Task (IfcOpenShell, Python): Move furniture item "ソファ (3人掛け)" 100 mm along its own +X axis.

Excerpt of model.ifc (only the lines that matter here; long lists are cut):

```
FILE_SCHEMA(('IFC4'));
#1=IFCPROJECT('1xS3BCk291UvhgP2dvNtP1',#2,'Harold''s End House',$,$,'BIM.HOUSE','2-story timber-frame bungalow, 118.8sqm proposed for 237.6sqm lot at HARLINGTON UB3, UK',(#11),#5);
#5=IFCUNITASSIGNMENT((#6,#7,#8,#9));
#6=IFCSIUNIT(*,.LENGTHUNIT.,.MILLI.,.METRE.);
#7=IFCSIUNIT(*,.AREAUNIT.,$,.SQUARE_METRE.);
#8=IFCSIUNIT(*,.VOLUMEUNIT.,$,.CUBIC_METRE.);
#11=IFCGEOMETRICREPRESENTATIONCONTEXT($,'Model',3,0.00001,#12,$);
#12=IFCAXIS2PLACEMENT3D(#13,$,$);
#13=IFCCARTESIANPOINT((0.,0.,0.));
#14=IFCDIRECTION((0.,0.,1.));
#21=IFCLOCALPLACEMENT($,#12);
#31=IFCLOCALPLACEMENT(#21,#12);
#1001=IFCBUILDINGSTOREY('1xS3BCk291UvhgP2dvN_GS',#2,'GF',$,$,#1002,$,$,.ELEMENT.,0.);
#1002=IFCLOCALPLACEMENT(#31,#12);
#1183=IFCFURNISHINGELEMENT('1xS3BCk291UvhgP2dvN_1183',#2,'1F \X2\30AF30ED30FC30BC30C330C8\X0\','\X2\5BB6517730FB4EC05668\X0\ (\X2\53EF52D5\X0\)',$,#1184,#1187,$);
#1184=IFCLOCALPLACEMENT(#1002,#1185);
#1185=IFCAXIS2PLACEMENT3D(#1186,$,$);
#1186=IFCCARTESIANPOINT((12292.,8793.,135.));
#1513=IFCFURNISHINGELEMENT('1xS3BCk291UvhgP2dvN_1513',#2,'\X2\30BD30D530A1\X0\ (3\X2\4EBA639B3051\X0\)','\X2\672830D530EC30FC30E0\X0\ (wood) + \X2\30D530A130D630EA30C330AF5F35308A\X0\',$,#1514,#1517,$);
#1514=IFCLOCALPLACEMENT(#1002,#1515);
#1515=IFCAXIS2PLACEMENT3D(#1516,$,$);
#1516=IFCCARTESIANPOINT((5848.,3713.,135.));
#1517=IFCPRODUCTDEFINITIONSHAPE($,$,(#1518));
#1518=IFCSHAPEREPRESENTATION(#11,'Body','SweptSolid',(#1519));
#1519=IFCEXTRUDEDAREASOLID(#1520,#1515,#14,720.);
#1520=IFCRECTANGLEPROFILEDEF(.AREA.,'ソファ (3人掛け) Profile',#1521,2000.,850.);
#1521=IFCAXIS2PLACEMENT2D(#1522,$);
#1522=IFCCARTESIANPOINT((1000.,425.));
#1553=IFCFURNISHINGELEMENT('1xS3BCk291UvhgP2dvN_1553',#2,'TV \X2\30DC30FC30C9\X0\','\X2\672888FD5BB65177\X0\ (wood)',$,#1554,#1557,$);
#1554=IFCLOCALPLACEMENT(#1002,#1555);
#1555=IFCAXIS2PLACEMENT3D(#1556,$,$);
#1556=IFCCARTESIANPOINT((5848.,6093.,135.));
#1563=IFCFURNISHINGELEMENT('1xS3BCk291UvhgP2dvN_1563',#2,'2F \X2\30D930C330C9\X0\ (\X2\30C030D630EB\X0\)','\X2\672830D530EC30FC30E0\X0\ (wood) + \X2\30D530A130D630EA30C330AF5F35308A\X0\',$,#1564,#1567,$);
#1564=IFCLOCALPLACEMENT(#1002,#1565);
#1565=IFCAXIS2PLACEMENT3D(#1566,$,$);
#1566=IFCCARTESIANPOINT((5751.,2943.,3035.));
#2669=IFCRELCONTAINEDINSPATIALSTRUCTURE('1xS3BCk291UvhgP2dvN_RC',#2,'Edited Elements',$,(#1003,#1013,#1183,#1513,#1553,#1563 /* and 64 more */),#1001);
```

```python
import ifcopenshell
import ifcopenshell.api.geometry
import ifcopenshell.util.placement

model = ifcopenshell.open("model.ifc")

item = model.by_id(1513)
matrix = ifcopenshell.util.placement.get_local_placement(item.ObjectPlacement)
matrix[:3, 3] += matrix[:3, 0] * 100.0
ifcopenshell.api.geometry.edit_object_placement(model, product=item, matrix=matrix, is_si=False)

print(ifcopenshell.util.placement.get_local_placement(item.ObjectPlacement).round(3) + 0.0)

model.write("model_updated.ifc")
```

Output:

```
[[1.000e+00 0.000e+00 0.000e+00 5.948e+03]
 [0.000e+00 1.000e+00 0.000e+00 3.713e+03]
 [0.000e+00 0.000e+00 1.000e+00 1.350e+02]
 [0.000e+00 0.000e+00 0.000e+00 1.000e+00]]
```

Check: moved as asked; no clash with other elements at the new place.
